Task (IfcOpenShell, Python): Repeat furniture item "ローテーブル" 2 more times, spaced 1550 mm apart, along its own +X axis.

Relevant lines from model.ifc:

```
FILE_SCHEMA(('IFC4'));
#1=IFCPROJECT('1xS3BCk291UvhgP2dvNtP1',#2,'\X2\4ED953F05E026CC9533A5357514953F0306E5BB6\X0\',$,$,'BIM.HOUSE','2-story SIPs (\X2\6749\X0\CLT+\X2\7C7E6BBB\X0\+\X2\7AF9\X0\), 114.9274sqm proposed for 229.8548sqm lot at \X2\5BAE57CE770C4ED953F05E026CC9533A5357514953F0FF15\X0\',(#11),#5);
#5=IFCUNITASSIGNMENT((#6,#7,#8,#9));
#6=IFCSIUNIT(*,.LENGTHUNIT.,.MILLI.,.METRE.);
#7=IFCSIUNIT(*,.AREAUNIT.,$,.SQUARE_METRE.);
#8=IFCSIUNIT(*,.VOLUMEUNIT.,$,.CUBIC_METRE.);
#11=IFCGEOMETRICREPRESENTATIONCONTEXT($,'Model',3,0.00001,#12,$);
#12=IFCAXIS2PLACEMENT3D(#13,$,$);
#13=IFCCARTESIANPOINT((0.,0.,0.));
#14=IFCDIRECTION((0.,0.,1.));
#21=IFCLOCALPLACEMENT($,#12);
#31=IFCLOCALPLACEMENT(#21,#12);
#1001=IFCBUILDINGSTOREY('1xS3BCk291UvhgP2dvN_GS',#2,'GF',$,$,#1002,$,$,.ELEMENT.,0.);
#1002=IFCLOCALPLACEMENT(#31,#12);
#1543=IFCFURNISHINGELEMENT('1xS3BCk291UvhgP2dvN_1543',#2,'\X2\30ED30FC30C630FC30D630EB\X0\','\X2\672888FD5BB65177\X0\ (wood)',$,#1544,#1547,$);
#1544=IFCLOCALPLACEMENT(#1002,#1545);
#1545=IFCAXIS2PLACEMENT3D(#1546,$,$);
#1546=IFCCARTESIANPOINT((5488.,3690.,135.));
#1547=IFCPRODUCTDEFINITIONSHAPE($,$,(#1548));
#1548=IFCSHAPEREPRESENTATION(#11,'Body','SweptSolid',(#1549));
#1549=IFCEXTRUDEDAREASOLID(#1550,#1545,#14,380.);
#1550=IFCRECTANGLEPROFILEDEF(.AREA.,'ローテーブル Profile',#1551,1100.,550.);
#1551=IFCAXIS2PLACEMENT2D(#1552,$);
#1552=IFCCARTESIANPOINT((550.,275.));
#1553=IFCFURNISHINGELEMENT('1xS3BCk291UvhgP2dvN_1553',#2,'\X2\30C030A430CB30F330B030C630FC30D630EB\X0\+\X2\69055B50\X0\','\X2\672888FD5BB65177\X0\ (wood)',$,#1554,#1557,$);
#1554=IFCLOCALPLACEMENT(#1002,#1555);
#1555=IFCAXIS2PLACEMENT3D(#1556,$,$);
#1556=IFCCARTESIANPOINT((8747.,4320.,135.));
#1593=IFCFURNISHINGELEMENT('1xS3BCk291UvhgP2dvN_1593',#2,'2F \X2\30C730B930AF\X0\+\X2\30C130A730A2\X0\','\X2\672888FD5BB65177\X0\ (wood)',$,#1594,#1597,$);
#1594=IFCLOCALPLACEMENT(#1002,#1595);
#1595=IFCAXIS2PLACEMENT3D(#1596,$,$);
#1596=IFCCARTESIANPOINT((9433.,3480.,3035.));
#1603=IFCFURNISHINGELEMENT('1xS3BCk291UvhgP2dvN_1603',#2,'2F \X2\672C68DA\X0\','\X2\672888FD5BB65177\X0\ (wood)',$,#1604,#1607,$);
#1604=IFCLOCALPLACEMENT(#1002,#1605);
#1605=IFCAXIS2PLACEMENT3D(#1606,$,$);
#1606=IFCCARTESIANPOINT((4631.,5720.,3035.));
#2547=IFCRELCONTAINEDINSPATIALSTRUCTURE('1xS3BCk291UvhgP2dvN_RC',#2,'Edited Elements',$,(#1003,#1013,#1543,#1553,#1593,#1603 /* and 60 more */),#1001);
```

```python
import ifcopenshell
import ifcopenshell.api.geometry
import ifcopenshell.api.root
import ifcopenshell.util.element
import ifcopenshell.util.placement

model = ifcopenshell.open("model.ifc")


def reuse_history(source, copy):
    """copy_class also copies each property set's owner history, people and application; keep the originals."""
    for rel in copy.IsDefinedBy:
        if rel.is_a("IfcRelDefinesByProperties") and (history := rel.RelatingPropertyDefinition.OwnerHistory):
            rel.RelatingPropertyDefinition.OwnerHistory = source.OwnerHistory
            ifcopenshell.util.element.remove_deep2(model, history)


source = model.by_guid("1xS3BCk291UvhgP2dvN_1543")
base = ifcopenshell.util.placement.get_local_placement(source.ObjectPlacement)
step = base[:3, 0] * 1550.0

for i in range(1, 3):
    copy = ifcopenshell.api.root.copy_class(model, product=source)
    copy.Representation = ifcopenshell.util.element.copy_deep(
        model, source.Representation, exclude=["IfcGeometricRepresentationContext", "IfcRepresentationMap"]
    )
    reuse_history(source, copy)
    matrix = base.copy()
    matrix[:3, 3] += i * step
    print("added at", matrix[:3, 3].round(3) + 0.0)
    ifcopenshell.api.geometry.edit_object_placement(model, product=copy, matrix=matrix, is_si=False)

model.write("model-out.ifc")
```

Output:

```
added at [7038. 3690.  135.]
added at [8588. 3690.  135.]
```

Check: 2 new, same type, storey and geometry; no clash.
